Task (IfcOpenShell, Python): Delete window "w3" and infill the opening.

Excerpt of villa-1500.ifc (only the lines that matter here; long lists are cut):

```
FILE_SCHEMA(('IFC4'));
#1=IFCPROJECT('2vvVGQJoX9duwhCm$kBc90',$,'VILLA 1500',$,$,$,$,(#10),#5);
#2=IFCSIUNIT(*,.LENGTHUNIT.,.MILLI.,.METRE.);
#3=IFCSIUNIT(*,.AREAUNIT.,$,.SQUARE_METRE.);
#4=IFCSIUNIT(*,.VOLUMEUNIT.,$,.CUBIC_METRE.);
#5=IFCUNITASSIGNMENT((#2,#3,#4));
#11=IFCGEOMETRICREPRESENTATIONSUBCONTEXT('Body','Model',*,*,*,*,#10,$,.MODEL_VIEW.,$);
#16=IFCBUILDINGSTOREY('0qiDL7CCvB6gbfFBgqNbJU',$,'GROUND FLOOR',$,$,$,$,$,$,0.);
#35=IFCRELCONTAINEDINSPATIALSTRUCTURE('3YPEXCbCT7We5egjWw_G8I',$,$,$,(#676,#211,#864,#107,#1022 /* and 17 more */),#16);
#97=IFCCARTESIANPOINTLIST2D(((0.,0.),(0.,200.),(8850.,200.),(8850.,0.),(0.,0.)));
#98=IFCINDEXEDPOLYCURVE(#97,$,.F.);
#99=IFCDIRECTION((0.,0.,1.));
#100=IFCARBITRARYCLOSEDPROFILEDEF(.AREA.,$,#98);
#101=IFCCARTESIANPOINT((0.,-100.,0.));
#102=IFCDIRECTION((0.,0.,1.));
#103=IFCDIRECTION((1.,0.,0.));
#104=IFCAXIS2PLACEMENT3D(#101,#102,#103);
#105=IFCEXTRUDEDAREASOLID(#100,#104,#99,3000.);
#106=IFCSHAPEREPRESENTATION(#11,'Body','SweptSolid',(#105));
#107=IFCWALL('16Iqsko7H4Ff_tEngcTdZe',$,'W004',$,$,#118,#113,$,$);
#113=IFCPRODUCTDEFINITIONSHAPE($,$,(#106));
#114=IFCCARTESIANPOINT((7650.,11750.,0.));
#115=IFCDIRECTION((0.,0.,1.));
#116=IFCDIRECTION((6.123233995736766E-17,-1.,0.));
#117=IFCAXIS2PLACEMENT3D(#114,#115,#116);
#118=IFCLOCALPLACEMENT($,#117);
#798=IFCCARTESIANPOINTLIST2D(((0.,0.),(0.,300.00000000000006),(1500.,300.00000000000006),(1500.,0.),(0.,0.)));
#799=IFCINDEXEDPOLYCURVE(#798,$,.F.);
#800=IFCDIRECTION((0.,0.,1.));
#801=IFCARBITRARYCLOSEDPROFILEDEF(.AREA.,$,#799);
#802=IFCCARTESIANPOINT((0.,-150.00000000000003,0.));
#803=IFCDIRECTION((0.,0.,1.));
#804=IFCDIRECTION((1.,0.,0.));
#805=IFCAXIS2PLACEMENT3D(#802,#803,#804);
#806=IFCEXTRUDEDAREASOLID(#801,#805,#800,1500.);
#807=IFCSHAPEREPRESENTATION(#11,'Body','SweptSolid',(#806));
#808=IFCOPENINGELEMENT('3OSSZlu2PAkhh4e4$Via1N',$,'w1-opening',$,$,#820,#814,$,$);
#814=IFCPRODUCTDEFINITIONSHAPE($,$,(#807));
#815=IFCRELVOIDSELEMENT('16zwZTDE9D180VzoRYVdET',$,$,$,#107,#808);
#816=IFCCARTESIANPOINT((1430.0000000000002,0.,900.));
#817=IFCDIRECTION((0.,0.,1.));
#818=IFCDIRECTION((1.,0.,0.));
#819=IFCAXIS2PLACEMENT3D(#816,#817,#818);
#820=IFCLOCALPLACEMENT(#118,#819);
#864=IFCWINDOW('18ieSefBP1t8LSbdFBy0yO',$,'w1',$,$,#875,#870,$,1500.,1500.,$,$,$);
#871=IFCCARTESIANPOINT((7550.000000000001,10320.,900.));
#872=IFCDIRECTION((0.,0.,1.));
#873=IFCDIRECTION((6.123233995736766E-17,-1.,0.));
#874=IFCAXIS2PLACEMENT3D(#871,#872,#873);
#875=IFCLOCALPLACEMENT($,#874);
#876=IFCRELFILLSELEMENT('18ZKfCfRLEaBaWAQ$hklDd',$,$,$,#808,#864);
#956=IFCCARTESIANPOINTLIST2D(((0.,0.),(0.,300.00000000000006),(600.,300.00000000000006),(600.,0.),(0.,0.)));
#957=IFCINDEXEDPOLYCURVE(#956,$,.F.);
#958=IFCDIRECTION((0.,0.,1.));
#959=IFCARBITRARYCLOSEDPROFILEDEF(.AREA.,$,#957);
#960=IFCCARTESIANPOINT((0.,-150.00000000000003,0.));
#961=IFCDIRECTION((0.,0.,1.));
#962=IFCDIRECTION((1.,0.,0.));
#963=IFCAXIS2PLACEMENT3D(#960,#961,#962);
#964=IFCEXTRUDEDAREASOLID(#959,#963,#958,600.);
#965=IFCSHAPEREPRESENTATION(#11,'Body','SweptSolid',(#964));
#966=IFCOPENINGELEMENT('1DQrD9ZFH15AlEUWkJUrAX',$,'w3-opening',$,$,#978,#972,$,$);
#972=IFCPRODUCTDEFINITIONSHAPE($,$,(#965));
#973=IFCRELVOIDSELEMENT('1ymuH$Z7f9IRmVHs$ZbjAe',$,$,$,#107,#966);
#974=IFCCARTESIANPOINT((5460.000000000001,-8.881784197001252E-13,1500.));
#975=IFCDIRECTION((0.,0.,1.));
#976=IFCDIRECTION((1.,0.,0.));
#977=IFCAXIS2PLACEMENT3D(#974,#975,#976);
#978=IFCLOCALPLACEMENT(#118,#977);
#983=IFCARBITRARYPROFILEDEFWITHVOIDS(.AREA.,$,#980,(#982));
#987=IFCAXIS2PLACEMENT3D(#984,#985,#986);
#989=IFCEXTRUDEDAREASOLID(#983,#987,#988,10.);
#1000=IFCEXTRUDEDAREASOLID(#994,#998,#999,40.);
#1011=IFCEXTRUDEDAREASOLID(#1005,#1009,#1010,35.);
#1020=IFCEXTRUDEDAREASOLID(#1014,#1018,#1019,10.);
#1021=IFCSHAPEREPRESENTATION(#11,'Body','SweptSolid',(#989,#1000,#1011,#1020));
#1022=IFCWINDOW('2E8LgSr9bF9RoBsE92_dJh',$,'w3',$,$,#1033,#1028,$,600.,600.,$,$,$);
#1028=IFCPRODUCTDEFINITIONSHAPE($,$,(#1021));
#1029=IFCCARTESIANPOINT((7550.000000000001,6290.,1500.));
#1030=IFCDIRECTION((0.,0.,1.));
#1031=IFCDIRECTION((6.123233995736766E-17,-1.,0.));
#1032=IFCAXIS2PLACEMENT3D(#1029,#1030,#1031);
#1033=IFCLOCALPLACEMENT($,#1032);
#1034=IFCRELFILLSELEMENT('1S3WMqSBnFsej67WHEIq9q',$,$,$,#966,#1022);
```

```python
import ifcopenshell
import ifcopenshell.api.feature
import ifcopenshell.api.root
import ifcopenshell.geom
import ifcopenshell.util.shape

model = ifcopenshell.open("villa-1500.ifc")
settings = ifcopenshell.geom.settings()


def volume(element):
    """Net volume in cubic metres, openings subtracted."""
    shape = ifcopenshell.geom.create_shape(settings, element)
    return ifcopenshell.util.shape.get_volume(shape.geometry)


window = model.by_guid("2E8LgSr9bF9RoBsE92_dJh")
opening = window.FillsVoids[0].RelatingOpeningElement
wall = opening.VoidsElements[0].RelatingBuildingElement
before = volume(wall)

ifcopenshell.api.root.remove_product(model, product=window)
ifcopenshell.api.feature.remove_feature(model, feature=opening)

after = volume(wall)

print(f"wall volume {before:.3f} -> {after:.3f} m3")

model.write("villa-1500_v2.ifc")
```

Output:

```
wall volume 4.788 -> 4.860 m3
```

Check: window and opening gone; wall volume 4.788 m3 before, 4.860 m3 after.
